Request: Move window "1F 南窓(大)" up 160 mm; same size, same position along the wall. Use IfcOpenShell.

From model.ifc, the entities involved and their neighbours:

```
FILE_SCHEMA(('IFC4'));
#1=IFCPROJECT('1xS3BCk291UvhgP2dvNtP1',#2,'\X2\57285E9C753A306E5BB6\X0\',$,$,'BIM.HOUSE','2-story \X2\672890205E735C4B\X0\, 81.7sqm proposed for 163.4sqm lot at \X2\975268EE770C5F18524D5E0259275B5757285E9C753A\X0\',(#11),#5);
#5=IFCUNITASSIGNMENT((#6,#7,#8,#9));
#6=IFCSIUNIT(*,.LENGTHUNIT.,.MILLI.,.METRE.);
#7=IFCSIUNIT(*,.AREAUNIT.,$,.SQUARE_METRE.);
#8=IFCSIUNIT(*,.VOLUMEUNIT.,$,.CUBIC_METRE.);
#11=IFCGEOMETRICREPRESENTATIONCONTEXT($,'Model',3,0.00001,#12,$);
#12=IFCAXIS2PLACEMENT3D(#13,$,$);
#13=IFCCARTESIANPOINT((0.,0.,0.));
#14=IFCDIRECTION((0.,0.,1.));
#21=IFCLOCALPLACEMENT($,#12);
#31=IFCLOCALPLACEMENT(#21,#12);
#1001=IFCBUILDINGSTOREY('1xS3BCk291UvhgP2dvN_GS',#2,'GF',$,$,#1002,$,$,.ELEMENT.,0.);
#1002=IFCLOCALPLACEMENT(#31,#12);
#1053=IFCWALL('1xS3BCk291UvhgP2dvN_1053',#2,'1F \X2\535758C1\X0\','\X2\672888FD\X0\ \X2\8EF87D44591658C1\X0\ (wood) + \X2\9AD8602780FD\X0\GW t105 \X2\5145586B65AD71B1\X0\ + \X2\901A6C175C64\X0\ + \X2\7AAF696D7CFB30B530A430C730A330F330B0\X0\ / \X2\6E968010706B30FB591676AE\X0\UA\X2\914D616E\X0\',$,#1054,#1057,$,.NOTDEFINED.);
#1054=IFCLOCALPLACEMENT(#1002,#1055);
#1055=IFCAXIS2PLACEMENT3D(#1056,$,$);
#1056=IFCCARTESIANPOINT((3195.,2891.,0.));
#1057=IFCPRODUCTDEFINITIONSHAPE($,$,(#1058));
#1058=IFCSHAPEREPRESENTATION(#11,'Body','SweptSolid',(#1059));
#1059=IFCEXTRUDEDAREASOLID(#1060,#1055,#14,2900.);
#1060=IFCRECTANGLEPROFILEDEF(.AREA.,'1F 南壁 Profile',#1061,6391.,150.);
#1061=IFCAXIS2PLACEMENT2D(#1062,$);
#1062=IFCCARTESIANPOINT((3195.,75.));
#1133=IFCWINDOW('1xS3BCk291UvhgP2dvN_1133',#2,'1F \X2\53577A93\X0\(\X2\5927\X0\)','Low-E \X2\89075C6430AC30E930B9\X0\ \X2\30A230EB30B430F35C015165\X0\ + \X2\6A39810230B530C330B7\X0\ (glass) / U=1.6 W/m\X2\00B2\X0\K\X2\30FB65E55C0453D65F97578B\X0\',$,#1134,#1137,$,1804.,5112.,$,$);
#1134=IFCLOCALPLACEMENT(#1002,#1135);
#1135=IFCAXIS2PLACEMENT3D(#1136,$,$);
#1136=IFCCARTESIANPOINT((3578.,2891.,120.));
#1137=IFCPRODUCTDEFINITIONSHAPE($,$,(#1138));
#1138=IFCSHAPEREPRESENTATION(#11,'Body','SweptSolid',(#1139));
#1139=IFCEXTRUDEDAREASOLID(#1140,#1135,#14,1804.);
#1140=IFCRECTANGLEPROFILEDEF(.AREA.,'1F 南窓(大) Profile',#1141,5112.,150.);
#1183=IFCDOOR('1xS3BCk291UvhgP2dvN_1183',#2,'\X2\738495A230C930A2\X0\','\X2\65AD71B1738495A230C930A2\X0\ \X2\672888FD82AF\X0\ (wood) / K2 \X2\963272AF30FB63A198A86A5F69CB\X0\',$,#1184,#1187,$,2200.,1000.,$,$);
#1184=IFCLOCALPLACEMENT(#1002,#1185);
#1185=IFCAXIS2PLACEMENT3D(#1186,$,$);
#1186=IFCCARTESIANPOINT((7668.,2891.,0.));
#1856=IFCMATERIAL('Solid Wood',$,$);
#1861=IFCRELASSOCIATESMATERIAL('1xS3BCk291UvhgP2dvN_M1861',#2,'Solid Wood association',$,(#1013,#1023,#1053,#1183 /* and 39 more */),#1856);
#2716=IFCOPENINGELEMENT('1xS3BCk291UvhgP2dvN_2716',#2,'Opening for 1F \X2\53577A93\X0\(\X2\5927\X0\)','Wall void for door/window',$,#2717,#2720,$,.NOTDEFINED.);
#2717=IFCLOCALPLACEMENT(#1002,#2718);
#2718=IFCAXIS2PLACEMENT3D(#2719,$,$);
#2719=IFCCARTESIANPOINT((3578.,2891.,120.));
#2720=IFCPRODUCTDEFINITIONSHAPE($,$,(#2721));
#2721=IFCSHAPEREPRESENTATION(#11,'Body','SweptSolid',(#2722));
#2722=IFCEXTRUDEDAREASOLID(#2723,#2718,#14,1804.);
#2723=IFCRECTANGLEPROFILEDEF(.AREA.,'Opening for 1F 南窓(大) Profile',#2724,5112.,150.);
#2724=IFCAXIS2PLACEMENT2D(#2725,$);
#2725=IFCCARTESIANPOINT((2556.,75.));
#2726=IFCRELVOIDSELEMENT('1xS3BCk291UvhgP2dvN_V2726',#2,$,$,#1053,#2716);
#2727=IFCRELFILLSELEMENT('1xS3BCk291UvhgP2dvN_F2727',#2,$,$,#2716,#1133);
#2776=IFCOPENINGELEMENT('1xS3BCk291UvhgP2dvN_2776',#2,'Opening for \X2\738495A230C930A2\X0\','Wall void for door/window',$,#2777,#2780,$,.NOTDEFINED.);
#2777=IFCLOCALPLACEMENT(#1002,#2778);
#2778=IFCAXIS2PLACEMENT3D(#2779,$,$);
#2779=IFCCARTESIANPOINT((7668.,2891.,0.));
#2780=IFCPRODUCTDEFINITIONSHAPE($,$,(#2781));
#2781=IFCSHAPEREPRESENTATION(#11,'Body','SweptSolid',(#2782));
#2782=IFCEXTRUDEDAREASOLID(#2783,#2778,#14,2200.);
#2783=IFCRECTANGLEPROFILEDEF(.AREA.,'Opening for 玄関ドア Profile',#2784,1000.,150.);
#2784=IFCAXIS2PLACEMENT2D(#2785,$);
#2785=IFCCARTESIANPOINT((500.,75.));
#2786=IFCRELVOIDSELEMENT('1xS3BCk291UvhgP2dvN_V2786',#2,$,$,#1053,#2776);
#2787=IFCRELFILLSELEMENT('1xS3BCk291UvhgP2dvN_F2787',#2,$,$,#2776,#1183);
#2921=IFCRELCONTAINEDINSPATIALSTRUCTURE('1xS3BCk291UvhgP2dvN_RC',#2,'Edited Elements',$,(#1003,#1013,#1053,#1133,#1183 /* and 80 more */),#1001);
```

```python
import numpy as np
import ifcopenshell
import ifcopenshell.api.geometry
import ifcopenshell.util.placement
import ifcopenshell.util.unit

model = ifcopenshell.open("model.ifc")
unit_scale = ifcopenshell.util.unit.calculate_unit_scale(model)

window = model.by_guid("1xS3BCk291UvhgP2dvN_1133")
opening = window.FillsVoids[0].RelatingOpeningElement
dz = 0.16 / unit_scale

shift = np.array([0.0, 0.0, dz])
# The window is not placed relative to its opening, so move both.
for product in (opening, window):
    matrix = ifcopenshell.util.placement.get_local_placement(product.ObjectPlacement)
    matrix[:3, 3] += shift
    ifcopenshell.api.geometry.edit_object_placement(model, product=product, matrix=matrix, is_si=False)

print(f"moved by {dz * unit_scale:+.3f} m")

model.write("model-out.ifc")
```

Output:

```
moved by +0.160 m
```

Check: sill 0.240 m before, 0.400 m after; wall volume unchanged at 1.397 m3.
